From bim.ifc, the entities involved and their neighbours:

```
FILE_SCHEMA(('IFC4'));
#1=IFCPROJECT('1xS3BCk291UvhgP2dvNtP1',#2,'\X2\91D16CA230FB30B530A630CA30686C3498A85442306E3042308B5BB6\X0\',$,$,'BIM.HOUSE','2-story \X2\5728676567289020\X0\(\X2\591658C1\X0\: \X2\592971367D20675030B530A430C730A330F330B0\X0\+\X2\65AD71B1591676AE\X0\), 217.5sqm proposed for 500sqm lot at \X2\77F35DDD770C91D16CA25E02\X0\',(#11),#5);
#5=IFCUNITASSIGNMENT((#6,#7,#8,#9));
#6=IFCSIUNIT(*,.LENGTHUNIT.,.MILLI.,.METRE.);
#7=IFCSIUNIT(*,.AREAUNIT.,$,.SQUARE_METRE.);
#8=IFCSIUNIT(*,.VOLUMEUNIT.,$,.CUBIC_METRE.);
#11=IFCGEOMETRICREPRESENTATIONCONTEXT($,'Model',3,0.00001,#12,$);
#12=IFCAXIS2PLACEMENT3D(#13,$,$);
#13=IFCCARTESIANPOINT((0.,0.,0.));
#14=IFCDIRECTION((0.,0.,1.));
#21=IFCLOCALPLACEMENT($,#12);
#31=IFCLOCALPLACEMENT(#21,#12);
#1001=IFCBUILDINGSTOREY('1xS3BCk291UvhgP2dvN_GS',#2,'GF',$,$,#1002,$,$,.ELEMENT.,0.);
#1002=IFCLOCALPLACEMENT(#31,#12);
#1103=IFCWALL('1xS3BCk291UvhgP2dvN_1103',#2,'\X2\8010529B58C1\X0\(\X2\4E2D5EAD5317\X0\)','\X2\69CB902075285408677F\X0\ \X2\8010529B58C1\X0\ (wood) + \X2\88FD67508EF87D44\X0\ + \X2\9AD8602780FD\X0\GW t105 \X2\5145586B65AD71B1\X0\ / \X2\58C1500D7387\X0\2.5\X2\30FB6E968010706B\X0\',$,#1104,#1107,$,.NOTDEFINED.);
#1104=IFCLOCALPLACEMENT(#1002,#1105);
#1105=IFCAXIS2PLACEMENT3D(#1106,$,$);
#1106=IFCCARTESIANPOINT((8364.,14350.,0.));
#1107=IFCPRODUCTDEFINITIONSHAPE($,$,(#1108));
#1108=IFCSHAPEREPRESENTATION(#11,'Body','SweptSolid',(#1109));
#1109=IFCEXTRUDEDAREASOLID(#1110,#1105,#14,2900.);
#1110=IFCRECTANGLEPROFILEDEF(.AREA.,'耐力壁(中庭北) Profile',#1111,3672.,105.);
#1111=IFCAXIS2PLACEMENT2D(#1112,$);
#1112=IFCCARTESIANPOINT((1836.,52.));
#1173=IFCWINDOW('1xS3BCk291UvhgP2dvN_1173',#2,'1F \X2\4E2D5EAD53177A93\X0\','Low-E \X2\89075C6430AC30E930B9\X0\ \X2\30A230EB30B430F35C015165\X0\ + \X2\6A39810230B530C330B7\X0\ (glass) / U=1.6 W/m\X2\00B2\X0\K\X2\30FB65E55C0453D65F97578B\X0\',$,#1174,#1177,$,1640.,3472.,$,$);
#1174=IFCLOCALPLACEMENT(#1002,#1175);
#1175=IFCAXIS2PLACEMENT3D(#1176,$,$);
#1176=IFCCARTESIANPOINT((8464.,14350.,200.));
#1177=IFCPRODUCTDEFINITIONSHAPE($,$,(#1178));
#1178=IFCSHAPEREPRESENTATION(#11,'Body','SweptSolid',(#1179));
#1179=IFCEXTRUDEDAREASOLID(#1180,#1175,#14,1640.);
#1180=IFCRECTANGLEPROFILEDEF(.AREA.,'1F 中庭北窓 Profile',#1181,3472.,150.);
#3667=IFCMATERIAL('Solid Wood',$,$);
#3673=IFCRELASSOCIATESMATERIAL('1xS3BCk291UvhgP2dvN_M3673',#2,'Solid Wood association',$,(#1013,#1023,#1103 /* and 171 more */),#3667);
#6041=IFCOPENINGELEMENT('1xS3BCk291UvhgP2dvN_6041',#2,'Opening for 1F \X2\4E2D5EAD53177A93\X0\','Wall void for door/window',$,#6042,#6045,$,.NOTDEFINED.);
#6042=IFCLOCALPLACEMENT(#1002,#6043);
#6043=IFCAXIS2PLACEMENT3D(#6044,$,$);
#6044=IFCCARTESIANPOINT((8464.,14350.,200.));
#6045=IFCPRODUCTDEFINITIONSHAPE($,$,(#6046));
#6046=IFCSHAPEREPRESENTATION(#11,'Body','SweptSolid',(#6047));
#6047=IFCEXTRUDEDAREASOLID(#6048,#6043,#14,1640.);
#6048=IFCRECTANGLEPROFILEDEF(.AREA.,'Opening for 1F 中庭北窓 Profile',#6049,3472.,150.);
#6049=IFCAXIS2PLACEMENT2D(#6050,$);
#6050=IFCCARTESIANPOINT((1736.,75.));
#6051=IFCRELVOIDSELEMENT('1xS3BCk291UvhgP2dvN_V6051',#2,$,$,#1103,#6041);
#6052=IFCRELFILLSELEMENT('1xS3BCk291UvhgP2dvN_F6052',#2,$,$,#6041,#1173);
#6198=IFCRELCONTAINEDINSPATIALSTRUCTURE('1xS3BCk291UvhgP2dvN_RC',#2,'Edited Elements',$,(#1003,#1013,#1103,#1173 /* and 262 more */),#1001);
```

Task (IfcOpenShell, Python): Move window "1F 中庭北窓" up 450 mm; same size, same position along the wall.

```python
import numpy as np
import ifcopenshell
import ifcopenshell.api.geometry
import ifcopenshell.util.placement
import ifcopenshell.util.unit

model = ifcopenshell.open("bim.ifc")
unit_scale = ifcopenshell.util.unit.calculate_unit_scale(model)

window = model.by_guid("1xS3BCk291UvhgP2dvN_1173")
opening = window.FillsVoids[0].RelatingOpeningElement
dz = 450.0

shift = np.array([0.0, 0.0, dz])
# The window is not placed relative to its opening, so move both.
for product in (opening, window):
    matrix = ifcopenshell.util.placement.get_local_placement(product.ObjectPlacement)
    matrix[:3, 3] += shift
    ifcopenshell.api.geometry.edit_object_placement(model, product=product, matrix=matrix, is_si=False)

print(f"moved by {dz * unit_scale:+.3f} m")

model.write("bim_rev.ifc")
```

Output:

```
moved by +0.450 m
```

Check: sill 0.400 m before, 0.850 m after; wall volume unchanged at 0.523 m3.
